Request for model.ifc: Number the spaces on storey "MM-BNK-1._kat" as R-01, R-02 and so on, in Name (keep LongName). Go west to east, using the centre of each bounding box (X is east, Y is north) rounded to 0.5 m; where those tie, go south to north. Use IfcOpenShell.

First a look at what the model holds.

```python
import ifcopenshell
import ifcopenshell.util.element
import ifcopenshell.util.placement

model = ifcopenshell.open("model.ifc")
print(model.schema)
storey = next(s for s in model.by_type("IfcBuildingStorey") if s.Name == "MM-BNK-1._kat")
spaces = [e for e in ifcopenshell.util.element.get_decomposition(storey) if e.is_a("IfcSpace")]
for e in sorted(spaces, key=lambda e: e.id()):
    origin = ifcopenshell.util.placement.get_local_placement(e.ObjectPlacement)[:3, 3]
    print(e.id(), e.Name, e.LongName, origin.round(2) + 0.0, sep=" | ")
```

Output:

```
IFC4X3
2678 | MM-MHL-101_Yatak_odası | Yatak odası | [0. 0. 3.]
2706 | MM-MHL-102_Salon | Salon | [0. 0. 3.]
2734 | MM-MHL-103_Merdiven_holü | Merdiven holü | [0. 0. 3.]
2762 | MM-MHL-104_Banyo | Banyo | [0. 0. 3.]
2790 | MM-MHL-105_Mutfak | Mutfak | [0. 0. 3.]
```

```python
import ifcopenshell
import ifcopenshell.geom
import ifcopenshell.util.element
import ifcopenshell.util.shape

model = ifcopenshell.open("model.ifc")
settings = ifcopenshell.geom.settings()
settings.set("use-world-coords", True)


def centre(element):
    shape = ifcopenshell.geom.create_shape(settings, element)
    return ifcopenshell.util.shape.get_bbox_centroid(shape.geometry)


storey = next(s for s in model.by_type("IfcBuildingStorey") if s.Name == "MM-BNK-1._kat")
spaces = [e for e in ifcopenshell.util.element.get_decomposition(storey) if e.is_a("IfcSpace")]

# Insertion points can sit at a corner or the storey origin, so sort by the geometry (in metres).
centres = {e: centre(e) for e in spaces}
spaces.sort(key=lambda e: (round(centres[e][0] / 0.5), centres[e][1]))

for i, e in enumerate(spaces, start=1):
    number = f"R-{i:02d}"
    e.Name = number
    print(e.id(), number)

model.write("model-out.ifc")
```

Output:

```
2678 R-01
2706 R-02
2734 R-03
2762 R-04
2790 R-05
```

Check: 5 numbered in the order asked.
